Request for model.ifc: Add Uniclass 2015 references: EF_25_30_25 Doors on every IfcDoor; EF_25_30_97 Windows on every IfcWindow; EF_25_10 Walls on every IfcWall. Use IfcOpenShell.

First a look at what the model holds.

```python
import ifcopenshell

model = ifcopenshell.open("model.ifc")
print(model.schema)
print("classifications:", [c.Name for c in model.by_type("IfcClassification")])
for ifc_class in ("IfcDoor", "IfcRoof", "IfcStair", "IfcWall", "IfcWindow"):
    print(ifc_class, len(model.by_type(ifc_class)))
```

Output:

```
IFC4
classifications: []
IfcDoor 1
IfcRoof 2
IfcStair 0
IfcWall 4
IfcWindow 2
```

```python
import ifcopenshell
import ifcopenshell.api.classification

model = ifcopenshell.open("model.ifc")

system = ifcopenshell.api.classification.add_classification(model, classification="Uniclass 2015")

codes = {
    "IfcDoor": ("EF_25_30_25", "Doors"),
    "IfcWindow": ("EF_25_30_97", "Windows"),
    "IfcWall": ("EF_25_10", "Walls"),
}
for ifc_class, (code, name) in codes.items():
    products = model.by_type(ifc_class)
    ifcopenshell.api.classification.add_reference(
        model, products=products, classification=system, identification=code, name=name
    )
    print(code, len(products))

model.write("model_v2.ifc")
```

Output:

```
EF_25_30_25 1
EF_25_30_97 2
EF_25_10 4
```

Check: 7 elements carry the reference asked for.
